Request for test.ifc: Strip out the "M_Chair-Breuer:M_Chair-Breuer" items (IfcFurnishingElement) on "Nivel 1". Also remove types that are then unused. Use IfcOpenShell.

First a look at what the model holds.

```python
import ifcopenshell
import ifcopenshell.util.element

model = ifcopenshell.open("test.ifc")
print(model.schema)
storey = next(s for s in model.by_type("IfcBuildingStorey") if s.Name == "Nivel 1")
furniture = [e for e in ifcopenshell.util.element.get_decomposition(storey) if e.is_a("IfcFurnishingElement")]
seen = {}
for e in furniture:
    element_type = ifcopenshell.util.element.get_type(e)
    name = element_type.Name if element_type not in (None, e) else None
    seen[name] = seen.get(name, 0) + 1
for name, count in sorted(seen.items(), key=str):
    print(count, "x", name)
```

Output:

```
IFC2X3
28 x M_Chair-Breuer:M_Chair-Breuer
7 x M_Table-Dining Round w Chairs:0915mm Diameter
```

```python
import ifcopenshell
import ifcopenshell.api.root
import ifcopenshell.util.element

model = ifcopenshell.open("test.ifc")

storey = next(s for s in model.by_type("IfcBuildingStorey") if s.Name == "Nivel 1")
furniture = [e for e in ifcopenshell.util.element.get_decomposition(storey) if e.is_a("IfcFurnishingElement")]
targets = [e for e in furniture if (t := ifcopenshell.util.element.get_type(e)) not in (None, e) and t.Name == "M_Chair-Breuer:M_Chair-Breuer"]
types = {ifcopenshell.util.element.get_type(e) for e in targets} - {None, *targets}

for e in targets:
    ifcopenshell.api.root.remove_product(model, product=e)
print(len(targets), "removed")

unused = [t for t in types if not ifcopenshell.util.element.get_types(t)]
for t in unused:
    ifcopenshell.api.root.remove_product(model, product=t)
print(len(unused), "unused types removed")

model.write("test_v2.ifc")
```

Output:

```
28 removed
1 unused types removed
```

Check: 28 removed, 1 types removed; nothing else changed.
